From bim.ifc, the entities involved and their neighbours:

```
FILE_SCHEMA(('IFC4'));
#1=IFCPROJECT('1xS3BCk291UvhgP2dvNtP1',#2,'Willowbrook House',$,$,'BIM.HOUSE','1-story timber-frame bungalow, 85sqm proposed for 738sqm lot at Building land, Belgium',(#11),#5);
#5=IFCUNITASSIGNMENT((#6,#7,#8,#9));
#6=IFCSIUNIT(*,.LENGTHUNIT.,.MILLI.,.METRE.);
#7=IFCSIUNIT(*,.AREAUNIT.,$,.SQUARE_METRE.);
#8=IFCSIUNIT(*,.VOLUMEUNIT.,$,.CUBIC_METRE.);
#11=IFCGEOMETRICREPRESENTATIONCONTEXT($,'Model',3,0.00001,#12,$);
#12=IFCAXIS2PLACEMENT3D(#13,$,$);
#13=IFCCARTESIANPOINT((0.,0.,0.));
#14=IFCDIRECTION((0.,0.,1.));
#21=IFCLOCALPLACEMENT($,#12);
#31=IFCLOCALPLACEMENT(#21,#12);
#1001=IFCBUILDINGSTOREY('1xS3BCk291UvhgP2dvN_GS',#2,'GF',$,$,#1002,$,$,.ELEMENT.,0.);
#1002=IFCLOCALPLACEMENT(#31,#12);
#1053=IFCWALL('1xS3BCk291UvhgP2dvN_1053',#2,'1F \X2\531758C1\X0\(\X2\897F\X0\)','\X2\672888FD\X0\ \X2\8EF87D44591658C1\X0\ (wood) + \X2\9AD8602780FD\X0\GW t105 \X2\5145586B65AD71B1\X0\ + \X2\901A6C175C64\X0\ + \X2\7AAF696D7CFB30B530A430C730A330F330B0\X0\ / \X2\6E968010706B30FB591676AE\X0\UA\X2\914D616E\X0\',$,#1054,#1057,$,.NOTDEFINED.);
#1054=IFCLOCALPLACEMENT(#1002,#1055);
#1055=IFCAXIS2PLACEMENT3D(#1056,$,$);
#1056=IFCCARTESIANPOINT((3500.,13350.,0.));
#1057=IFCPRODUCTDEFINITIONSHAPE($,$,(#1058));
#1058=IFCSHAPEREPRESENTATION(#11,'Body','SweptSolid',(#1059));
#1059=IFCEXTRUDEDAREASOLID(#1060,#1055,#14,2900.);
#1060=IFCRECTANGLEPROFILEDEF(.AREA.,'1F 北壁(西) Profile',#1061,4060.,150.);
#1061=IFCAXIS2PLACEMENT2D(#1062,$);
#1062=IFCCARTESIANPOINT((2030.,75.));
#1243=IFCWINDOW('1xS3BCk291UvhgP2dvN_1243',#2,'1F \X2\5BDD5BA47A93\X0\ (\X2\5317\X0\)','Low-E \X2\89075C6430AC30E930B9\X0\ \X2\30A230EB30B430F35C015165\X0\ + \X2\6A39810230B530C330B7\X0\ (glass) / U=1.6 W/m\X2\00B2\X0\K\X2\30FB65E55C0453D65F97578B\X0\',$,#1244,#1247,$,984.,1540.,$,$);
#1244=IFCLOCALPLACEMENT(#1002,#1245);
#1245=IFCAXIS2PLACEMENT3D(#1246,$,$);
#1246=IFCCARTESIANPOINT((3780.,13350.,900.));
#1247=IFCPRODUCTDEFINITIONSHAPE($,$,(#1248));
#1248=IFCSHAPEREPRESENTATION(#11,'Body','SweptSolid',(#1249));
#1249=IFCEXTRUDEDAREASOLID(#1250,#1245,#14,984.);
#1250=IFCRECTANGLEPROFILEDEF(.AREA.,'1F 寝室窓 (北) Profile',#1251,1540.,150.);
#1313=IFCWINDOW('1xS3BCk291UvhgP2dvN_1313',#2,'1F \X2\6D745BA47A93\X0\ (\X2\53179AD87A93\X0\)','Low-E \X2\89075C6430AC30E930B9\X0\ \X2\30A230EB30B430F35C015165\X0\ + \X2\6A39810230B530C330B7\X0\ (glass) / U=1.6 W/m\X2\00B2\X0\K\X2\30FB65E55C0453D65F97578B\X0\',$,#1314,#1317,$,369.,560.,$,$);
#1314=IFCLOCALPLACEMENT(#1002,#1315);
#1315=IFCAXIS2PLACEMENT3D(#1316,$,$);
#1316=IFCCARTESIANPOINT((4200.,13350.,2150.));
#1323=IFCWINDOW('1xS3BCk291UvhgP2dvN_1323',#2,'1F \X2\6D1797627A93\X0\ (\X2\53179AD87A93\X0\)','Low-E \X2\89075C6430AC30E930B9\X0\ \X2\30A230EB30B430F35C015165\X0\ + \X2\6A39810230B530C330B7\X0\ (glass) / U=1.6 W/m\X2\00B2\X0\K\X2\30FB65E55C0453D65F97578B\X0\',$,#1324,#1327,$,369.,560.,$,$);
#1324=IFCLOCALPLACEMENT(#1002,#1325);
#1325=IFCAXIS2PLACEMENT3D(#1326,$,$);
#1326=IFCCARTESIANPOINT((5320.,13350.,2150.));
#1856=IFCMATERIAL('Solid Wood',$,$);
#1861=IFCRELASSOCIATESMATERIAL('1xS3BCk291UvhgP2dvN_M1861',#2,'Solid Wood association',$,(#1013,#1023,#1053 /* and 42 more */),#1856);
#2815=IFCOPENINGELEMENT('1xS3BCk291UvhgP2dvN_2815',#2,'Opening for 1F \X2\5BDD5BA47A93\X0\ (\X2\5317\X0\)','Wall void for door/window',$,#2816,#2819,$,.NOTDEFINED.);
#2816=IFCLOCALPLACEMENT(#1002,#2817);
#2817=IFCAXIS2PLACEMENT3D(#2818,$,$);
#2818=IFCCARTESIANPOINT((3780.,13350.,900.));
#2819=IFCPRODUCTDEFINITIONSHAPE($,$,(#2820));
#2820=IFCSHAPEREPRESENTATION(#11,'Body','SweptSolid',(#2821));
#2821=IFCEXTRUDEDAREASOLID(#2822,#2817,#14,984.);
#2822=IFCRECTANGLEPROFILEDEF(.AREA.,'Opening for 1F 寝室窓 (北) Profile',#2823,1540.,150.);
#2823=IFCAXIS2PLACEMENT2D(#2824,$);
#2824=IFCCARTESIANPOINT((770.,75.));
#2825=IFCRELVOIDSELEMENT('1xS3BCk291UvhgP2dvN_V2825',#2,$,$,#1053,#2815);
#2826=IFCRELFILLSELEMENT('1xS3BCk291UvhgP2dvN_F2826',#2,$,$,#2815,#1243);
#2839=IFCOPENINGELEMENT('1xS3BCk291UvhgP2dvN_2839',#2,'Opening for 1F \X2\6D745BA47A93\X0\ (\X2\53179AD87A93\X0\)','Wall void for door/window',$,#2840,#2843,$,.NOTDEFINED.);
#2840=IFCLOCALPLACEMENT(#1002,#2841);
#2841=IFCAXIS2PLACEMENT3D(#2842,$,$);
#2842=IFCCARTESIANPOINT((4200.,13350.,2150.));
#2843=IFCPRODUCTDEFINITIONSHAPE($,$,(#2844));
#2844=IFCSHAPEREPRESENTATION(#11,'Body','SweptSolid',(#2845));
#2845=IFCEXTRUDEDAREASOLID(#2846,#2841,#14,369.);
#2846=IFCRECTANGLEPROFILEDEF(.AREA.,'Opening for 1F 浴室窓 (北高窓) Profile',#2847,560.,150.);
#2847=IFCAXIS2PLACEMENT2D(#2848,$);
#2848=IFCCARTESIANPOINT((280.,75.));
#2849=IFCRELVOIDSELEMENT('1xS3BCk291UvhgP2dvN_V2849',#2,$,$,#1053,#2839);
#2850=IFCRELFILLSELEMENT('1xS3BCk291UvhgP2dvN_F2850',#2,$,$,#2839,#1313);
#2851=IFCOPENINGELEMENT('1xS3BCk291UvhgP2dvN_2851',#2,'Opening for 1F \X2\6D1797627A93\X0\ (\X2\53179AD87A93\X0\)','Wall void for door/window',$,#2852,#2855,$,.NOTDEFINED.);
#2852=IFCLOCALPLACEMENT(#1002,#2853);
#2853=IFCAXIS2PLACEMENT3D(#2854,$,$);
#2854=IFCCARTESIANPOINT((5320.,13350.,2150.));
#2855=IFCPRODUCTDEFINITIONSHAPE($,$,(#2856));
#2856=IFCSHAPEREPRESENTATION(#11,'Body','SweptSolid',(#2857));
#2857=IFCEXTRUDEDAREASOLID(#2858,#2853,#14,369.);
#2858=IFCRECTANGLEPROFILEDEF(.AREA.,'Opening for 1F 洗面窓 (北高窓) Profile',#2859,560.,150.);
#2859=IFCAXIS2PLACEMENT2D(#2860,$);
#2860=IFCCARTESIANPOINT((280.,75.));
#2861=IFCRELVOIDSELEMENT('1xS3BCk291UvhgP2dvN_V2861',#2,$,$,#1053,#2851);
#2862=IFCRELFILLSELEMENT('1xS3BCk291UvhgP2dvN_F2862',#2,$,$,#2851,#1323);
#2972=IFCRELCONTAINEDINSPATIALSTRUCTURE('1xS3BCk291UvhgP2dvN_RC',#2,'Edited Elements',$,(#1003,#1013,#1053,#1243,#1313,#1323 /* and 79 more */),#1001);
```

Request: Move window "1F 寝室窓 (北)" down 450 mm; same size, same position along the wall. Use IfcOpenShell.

```python
import numpy as np
import ifcopenshell
import ifcopenshell.api.geometry
import ifcopenshell.util.placement
import ifcopenshell.util.unit

model = ifcopenshell.open("bim.ifc")
unit_scale = ifcopenshell.util.unit.calculate_unit_scale(model)

window = model.by_id(1243)
opening = window.FillsVoids[0].RelatingOpeningElement
dz = -450.0

shift = np.array([0.0, 0.0, dz])
# The window is not placed relative to its opening, so move both.
for product in (opening, window):
    matrix = ifcopenshell.util.placement.get_local_placement(product.ObjectPlacement)
    matrix[:3, 3] += shift
    ifcopenshell.api.geometry.edit_object_placement(model, product=product, matrix=matrix, is_si=False)

print(f"moved by {dz * unit_scale:+.3f} m")

model.write("bim-out.ifc")
```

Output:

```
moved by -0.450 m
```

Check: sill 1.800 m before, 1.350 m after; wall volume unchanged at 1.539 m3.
